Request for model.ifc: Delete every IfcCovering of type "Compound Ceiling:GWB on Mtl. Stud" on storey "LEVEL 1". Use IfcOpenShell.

First a look at what the model holds.

```python
import ifcopenshell
import ifcopenshell.util.element

model = ifcopenshell.open("model.ifc")
print(model.schema)
storey = next(s for s in model.by_type("IfcBuildingStorey") if s.Name == "LEVEL 1")
coverings = [e for e in ifcopenshell.util.element.get_decomposition(storey) if e.is_a("IfcCovering")]
seen = {}
for e in coverings:
    element_type = ifcopenshell.util.element.get_type(e)
    name = element_type.Name if element_type not in (None, e) else None
    seen[name] = seen.get(name, 0) + 1
for name, count in sorted(seen.items(), key=str):
    print(count, "x", name)
```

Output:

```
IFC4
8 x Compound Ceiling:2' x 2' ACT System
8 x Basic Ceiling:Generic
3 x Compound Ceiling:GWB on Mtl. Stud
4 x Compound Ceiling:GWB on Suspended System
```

```python
import ifcopenshell
import ifcopenshell.api.root
import ifcopenshell.util.element

model = ifcopenshell.open("model.ifc")

storey = next(s for s in model.by_type("IfcBuildingStorey") if s.Name == "LEVEL 1")
coverings = [e for e in ifcopenshell.util.element.get_decomposition(storey) if e.is_a("IfcCovering")]
targets = [e for e in coverings if (t := ifcopenshell.util.element.get_type(e)) not in (None, e) and t.Name == "Compound Ceiling:GWB on Mtl. Stud"]

for e in targets:
    ifcopenshell.api.root.remove_product(model, product=e)
print(len(targets), "removed")

model.write("model_v2.ifc")
```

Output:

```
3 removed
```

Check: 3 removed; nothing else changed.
